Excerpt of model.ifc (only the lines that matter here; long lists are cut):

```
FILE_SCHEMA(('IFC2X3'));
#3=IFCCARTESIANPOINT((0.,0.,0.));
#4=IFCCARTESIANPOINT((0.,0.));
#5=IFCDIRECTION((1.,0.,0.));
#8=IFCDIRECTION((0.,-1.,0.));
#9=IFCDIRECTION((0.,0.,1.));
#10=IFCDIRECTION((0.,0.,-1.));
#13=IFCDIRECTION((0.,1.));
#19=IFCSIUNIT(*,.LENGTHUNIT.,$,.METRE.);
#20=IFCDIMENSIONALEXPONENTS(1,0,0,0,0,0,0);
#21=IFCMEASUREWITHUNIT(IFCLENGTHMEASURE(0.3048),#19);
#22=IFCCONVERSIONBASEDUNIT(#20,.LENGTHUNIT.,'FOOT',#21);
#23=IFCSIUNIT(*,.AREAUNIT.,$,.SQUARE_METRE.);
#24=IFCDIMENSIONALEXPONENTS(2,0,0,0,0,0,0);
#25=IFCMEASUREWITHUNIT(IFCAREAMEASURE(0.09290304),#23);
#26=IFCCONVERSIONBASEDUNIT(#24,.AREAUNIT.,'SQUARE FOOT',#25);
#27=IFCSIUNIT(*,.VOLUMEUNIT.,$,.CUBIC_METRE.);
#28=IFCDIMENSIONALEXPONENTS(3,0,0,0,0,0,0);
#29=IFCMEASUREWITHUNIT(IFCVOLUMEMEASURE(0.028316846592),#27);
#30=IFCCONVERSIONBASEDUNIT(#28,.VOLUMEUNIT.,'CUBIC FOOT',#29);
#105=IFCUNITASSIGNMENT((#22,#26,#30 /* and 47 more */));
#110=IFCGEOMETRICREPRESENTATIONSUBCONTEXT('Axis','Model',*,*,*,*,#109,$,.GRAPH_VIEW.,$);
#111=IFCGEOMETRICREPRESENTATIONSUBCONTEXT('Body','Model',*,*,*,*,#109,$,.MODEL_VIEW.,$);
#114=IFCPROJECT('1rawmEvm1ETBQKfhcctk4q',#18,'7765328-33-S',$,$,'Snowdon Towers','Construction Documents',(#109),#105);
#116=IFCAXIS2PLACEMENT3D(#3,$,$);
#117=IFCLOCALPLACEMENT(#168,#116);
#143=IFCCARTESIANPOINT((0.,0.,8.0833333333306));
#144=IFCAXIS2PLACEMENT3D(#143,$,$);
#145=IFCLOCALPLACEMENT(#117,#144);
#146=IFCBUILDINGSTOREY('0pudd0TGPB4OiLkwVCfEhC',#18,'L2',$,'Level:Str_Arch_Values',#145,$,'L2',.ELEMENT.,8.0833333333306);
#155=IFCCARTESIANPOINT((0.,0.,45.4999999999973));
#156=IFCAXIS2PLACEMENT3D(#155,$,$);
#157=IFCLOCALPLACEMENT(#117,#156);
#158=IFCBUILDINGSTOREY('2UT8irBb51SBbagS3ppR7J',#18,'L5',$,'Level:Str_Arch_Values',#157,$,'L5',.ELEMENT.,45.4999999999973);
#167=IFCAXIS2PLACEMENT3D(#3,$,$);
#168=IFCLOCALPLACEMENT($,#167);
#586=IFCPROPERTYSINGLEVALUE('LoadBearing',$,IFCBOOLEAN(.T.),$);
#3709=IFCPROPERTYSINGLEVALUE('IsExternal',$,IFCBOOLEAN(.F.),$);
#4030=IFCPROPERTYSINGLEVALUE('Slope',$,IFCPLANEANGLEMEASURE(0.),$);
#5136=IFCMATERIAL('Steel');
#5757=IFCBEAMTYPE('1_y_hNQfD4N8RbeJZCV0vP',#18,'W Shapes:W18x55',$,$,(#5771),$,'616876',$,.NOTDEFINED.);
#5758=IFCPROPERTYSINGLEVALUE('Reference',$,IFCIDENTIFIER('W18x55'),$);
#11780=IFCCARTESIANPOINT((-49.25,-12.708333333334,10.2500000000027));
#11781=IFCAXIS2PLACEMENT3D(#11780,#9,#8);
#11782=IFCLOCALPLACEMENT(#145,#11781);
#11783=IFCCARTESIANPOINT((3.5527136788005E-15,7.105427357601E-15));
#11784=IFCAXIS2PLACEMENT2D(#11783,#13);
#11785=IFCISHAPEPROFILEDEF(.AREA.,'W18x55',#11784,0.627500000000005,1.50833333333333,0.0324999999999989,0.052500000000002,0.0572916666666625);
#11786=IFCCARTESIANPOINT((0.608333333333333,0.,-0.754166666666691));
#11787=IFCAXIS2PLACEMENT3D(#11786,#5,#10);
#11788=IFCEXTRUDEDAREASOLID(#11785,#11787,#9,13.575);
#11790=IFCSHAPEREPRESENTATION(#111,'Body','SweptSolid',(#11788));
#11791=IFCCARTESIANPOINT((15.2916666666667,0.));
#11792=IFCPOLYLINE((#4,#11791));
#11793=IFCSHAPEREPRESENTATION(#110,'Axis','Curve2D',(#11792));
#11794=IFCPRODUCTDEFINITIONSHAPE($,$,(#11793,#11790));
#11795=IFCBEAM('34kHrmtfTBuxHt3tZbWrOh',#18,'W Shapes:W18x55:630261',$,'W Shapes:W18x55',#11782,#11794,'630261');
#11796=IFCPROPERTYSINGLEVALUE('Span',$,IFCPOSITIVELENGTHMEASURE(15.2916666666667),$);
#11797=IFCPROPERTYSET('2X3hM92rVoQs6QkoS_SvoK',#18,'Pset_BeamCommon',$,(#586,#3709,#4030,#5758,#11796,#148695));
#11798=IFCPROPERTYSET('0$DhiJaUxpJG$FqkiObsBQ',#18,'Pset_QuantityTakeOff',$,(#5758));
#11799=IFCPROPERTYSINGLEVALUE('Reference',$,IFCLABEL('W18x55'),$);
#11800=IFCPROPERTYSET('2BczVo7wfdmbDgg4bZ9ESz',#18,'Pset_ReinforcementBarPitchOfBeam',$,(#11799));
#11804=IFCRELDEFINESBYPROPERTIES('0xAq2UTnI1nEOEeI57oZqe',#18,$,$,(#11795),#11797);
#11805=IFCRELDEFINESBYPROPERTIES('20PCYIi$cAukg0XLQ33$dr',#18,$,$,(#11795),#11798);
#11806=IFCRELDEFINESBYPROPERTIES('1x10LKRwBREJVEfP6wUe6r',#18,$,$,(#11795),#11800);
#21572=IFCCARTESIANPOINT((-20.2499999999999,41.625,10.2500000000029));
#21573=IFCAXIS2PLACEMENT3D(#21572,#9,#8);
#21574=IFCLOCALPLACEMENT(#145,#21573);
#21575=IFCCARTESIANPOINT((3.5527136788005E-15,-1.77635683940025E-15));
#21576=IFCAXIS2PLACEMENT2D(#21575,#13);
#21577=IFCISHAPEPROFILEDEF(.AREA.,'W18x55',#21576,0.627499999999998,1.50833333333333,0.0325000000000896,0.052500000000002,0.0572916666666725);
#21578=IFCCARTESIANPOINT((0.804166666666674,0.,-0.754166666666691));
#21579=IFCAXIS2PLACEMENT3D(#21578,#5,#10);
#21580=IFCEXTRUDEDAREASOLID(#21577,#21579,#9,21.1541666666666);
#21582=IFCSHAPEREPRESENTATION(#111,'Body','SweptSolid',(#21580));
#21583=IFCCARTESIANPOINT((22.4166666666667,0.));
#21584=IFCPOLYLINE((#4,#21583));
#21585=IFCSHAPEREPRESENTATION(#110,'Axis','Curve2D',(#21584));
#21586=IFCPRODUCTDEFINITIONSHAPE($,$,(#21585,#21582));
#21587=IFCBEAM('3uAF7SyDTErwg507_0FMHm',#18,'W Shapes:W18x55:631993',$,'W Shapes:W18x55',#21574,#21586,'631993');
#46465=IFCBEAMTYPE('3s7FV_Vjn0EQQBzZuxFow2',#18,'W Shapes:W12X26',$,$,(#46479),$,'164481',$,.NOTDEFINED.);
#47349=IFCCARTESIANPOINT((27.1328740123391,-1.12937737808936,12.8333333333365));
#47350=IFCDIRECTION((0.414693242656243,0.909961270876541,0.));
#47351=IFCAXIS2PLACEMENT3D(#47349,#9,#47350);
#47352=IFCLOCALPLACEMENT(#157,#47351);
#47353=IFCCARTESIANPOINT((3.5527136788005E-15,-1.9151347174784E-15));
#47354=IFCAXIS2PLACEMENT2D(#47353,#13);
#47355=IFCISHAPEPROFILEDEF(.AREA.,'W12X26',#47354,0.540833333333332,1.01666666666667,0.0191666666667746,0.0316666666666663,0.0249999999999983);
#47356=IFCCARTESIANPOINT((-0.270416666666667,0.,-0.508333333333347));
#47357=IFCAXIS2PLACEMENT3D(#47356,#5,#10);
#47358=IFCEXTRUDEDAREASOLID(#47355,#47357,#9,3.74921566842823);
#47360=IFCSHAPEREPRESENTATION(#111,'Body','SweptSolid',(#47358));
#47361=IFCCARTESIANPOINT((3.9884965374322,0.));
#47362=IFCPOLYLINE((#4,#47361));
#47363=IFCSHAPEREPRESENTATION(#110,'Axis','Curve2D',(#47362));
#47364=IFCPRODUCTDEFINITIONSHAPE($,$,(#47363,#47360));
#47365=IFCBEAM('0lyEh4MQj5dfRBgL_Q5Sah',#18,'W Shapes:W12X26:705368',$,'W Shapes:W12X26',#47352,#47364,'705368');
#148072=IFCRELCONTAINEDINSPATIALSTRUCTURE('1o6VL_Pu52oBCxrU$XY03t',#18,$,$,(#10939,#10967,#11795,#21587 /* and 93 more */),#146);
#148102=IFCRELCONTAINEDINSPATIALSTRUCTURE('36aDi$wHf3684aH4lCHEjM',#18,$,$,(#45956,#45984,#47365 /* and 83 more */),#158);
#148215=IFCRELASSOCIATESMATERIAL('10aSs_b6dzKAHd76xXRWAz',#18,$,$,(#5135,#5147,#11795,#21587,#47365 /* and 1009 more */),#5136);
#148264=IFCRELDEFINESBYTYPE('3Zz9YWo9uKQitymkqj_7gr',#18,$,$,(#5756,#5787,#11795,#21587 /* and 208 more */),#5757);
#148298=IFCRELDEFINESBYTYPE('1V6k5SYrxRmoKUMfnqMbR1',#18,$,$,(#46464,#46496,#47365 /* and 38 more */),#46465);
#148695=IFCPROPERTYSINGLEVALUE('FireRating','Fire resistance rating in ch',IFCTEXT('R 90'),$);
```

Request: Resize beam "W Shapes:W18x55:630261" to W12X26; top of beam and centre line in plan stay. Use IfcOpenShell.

```python
import ifcopenshell
import ifcopenshell.api.pset
import ifcopenshell.api.type
import ifcopenshell.util.element
import ifcopenshell.util.representation

model = ifcopenshell.open("model.ifc")

member = model.by_id(11795)
source = next(p for p in model.by_type("IfcIShapeProfileDef") if p.ProfileName == "W12X26")

body = ifcopenshell.util.representation.get_representation(member, "Model", "Body")
solid = body.Items[0]
old_profile = solid.SweptArea

# Copy the section's sizes but keep this member's own profile position.
profile = ifcopenshell.util.element.copy(model, source)
# Profiles are centred, so shift by half the change in depth to hold the top.
shift = (old_profile.OverallDepth - profile.OverallDepth) / 2
x, y = old_profile.Position.Location.Coordinates
up = (-1.0, 0.0)  # upwards, in the solid's own plane
location = model.createIfcCartesianPoint((x + up[0] * shift, y + up[1] * shift))
profile.Position = model.createIfcAxis2Placement2D(location, old_profile.Position.RefDirection)
solid.SweptArea = profile
if not model.get_total_inverses(old_profile):
    ifcopenshell.util.element.remove_deep2(model, old_profile)

new_type = model.by_guid("3s7FV_Vjn0EQQBzZuxFow2")
ifcopenshell.api.type.assign_type(
    model, related_objects=[member], relating_type=new_type, should_map_representations=False
)
member.Name = member.Name.replace("W18x55", "W12X26")
member.ObjectType = "W Shapes:W12X26"
pset = model.by_id(ifcopenshell.util.element.get_pset(member, "Pset_BeamCommon", should_inherit=False)["id"])
ifcopenshell.api.pset.edit_pset(model, pset=pset, properties={"Reference": "W12X26"})
pset = model.by_id(ifcopenshell.util.element.get_pset(member, "Pset_QuantityTakeOff", should_inherit=False)["id"])
ifcopenshell.api.pset.edit_pset(model, pset=pset, properties={"Reference": "W12X26"})
pset = model.by_id(ifcopenshell.util.element.get_pset(member, "Pset_ReinforcementBarPitchOfBeam", should_inherit=False)["id"])
ifcopenshell.api.pset.edit_pset(model, pset=pset, properties={"Reference": "W12X26"})

print(solid.SweptArea)

model.write("model_edited.ifc")
```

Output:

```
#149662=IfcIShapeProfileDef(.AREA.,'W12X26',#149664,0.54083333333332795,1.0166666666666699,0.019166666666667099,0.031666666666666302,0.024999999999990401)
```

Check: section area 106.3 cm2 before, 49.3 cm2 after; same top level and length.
